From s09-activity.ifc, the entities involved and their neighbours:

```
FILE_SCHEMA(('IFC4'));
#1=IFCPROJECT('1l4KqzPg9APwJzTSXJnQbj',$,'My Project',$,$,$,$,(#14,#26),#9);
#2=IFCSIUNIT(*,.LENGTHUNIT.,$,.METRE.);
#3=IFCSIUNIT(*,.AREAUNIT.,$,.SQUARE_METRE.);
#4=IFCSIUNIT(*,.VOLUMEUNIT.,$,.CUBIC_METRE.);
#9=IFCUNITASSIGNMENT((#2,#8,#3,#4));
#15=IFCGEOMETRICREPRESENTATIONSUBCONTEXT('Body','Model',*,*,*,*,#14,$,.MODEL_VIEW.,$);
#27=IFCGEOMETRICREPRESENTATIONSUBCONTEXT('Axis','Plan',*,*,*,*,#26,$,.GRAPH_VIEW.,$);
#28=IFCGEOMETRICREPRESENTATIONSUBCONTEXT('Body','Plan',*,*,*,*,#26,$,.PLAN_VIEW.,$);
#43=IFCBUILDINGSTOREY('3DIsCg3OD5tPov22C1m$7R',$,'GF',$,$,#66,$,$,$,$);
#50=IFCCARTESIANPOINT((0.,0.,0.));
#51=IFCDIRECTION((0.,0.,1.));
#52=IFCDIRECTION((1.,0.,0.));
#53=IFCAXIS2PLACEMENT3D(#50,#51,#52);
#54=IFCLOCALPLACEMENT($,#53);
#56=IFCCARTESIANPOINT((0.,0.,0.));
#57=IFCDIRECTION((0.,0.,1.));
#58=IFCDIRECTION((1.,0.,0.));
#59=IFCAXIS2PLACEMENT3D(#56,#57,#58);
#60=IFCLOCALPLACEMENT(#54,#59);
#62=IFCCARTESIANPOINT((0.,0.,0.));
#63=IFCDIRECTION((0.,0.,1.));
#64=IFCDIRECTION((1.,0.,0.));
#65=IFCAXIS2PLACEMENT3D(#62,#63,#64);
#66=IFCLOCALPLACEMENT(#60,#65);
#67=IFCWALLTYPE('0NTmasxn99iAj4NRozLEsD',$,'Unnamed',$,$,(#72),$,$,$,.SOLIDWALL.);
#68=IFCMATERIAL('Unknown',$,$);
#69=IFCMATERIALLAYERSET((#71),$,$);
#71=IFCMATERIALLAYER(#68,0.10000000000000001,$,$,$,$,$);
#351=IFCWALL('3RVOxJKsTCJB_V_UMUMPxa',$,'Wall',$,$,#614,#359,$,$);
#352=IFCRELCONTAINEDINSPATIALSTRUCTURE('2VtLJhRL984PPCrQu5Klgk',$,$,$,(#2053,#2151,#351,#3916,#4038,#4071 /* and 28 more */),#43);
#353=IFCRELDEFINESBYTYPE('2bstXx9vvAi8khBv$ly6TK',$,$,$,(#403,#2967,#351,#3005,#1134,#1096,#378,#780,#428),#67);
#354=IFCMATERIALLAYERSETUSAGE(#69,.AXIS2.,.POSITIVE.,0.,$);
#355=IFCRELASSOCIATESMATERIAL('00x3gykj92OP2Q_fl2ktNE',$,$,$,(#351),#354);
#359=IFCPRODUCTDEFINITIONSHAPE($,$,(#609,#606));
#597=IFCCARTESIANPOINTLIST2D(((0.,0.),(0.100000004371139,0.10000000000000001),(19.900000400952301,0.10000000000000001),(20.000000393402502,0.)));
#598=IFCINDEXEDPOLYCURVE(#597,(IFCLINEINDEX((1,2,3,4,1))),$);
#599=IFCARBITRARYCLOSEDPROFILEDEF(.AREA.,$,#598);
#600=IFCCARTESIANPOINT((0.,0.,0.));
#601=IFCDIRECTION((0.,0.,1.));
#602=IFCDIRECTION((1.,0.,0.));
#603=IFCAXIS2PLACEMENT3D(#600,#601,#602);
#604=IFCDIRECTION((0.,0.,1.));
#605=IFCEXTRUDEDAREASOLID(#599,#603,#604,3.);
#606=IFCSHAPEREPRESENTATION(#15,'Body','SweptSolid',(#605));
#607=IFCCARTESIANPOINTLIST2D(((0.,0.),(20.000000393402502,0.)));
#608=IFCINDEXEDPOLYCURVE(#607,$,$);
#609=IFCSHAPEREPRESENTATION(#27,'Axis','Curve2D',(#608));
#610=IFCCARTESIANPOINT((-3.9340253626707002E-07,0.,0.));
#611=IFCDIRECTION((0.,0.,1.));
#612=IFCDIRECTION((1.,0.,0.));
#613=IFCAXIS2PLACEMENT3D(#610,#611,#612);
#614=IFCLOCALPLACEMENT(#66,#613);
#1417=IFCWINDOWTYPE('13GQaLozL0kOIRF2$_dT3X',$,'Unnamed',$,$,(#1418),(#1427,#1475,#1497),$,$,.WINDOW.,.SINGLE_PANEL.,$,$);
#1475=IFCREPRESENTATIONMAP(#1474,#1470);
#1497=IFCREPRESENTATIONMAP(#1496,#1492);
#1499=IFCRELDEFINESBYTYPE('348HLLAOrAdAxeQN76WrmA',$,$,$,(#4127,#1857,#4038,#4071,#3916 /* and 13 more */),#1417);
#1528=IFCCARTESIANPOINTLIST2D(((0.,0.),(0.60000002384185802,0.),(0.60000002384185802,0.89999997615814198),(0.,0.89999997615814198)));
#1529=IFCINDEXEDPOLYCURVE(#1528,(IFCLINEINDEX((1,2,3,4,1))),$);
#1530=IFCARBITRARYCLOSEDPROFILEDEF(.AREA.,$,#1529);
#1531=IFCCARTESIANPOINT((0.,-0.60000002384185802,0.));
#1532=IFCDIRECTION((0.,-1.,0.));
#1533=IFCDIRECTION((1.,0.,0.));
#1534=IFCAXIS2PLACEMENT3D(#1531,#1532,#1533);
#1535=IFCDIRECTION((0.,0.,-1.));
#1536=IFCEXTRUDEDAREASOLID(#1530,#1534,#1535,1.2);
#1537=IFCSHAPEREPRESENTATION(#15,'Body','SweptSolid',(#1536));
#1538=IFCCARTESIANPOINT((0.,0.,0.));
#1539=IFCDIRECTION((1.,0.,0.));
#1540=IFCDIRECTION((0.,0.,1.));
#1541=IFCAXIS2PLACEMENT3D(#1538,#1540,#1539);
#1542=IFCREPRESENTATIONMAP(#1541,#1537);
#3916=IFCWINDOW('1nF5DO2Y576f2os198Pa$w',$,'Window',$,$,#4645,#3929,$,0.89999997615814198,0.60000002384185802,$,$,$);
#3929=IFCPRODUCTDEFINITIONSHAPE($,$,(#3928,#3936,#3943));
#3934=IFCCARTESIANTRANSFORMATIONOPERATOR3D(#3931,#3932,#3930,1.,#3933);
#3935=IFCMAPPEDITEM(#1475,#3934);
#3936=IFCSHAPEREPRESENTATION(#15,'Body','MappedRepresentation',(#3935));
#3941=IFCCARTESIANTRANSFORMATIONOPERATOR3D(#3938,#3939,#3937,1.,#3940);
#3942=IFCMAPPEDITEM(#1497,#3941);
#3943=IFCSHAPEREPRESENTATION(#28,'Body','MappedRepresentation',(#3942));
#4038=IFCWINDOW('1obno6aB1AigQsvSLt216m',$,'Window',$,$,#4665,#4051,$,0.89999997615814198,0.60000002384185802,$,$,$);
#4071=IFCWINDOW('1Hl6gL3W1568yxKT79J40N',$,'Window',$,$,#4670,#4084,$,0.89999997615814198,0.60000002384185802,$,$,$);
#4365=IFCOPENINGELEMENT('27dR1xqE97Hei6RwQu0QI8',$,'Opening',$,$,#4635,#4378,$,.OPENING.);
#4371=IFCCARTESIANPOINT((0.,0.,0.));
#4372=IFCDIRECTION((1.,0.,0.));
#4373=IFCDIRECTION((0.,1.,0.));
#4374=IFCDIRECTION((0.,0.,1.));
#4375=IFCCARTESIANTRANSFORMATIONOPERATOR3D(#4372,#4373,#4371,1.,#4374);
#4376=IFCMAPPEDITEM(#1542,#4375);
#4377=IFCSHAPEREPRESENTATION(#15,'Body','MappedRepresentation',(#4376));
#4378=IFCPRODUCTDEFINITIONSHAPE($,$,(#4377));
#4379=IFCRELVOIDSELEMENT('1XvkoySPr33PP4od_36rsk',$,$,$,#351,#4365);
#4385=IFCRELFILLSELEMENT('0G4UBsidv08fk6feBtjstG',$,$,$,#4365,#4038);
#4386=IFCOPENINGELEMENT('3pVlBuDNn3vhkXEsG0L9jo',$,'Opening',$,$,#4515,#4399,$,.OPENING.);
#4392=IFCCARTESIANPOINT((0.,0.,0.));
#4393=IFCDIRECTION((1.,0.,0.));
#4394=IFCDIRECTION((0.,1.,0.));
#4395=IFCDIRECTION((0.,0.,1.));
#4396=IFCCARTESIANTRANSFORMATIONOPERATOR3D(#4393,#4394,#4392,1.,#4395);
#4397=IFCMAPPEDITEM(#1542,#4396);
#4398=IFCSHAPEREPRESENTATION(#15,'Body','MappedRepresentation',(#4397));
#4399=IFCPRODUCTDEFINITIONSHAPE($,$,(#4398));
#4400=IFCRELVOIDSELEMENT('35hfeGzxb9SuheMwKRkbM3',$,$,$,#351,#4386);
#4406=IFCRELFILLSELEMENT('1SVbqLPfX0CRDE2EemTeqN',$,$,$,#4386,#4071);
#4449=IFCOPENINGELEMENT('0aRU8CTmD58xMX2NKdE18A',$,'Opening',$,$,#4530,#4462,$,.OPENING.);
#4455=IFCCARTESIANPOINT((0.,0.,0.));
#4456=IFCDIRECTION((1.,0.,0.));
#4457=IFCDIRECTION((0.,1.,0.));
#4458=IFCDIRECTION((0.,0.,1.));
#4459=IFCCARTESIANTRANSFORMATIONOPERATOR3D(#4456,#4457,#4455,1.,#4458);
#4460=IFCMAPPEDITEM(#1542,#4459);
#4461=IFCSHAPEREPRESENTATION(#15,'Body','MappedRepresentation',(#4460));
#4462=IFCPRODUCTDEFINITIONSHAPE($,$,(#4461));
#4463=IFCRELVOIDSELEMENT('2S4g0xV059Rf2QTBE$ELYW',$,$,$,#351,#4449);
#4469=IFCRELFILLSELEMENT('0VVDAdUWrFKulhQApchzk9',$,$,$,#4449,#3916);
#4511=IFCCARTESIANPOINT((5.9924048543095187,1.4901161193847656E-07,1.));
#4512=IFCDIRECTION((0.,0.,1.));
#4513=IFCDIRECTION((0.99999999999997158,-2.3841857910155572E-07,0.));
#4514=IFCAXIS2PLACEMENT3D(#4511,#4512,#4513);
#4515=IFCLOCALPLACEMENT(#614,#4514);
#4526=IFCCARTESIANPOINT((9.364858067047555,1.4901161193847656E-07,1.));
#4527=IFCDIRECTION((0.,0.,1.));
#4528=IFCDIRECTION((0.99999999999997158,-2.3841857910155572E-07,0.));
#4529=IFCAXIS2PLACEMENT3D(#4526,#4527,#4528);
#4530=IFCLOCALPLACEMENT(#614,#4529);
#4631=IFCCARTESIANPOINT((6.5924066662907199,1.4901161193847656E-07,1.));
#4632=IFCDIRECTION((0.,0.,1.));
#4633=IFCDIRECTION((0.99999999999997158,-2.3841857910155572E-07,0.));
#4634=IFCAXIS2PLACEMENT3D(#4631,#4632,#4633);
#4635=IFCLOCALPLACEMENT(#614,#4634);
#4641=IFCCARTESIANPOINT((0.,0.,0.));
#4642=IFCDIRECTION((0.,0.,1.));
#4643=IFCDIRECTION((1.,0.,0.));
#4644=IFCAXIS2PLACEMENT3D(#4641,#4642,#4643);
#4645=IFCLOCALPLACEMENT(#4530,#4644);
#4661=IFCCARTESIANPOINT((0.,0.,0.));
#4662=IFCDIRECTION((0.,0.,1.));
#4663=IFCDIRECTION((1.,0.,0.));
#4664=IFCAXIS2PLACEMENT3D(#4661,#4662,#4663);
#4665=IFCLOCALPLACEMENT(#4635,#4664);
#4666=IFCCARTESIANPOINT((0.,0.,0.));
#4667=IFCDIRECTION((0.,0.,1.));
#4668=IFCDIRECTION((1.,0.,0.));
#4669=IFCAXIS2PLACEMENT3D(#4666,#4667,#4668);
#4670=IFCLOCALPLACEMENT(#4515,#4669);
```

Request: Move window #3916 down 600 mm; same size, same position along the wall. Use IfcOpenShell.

```python
import numpy as np
import ifcopenshell
import ifcopenshell.api.geometry
import ifcopenshell.util.placement
import ifcopenshell.util.unit

model = ifcopenshell.open("s09-activity.ifc")
unit_scale = ifcopenshell.util.unit.calculate_unit_scale(model)

window = model.by_id(3916)
opening = window.FillsVoids[0].RelatingOpeningElement
dz = -0.6 / unit_scale

shift = np.array([0.0, 0.0, dz])
# The window is placed relative to its opening, so it follows when the opening moves.
matrix = ifcopenshell.util.placement.get_local_placement(opening.ObjectPlacement)
matrix[:3, 3] += shift
ifcopenshell.api.geometry.edit_object_placement(
    model, product=opening, matrix=matrix, is_si=False, should_transform_children=True
)

print(f"moved by {dz * unit_scale:+.3f} m")

model.write("s09-activity-out.ifc")
```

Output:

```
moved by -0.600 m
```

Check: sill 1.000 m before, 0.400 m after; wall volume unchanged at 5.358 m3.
